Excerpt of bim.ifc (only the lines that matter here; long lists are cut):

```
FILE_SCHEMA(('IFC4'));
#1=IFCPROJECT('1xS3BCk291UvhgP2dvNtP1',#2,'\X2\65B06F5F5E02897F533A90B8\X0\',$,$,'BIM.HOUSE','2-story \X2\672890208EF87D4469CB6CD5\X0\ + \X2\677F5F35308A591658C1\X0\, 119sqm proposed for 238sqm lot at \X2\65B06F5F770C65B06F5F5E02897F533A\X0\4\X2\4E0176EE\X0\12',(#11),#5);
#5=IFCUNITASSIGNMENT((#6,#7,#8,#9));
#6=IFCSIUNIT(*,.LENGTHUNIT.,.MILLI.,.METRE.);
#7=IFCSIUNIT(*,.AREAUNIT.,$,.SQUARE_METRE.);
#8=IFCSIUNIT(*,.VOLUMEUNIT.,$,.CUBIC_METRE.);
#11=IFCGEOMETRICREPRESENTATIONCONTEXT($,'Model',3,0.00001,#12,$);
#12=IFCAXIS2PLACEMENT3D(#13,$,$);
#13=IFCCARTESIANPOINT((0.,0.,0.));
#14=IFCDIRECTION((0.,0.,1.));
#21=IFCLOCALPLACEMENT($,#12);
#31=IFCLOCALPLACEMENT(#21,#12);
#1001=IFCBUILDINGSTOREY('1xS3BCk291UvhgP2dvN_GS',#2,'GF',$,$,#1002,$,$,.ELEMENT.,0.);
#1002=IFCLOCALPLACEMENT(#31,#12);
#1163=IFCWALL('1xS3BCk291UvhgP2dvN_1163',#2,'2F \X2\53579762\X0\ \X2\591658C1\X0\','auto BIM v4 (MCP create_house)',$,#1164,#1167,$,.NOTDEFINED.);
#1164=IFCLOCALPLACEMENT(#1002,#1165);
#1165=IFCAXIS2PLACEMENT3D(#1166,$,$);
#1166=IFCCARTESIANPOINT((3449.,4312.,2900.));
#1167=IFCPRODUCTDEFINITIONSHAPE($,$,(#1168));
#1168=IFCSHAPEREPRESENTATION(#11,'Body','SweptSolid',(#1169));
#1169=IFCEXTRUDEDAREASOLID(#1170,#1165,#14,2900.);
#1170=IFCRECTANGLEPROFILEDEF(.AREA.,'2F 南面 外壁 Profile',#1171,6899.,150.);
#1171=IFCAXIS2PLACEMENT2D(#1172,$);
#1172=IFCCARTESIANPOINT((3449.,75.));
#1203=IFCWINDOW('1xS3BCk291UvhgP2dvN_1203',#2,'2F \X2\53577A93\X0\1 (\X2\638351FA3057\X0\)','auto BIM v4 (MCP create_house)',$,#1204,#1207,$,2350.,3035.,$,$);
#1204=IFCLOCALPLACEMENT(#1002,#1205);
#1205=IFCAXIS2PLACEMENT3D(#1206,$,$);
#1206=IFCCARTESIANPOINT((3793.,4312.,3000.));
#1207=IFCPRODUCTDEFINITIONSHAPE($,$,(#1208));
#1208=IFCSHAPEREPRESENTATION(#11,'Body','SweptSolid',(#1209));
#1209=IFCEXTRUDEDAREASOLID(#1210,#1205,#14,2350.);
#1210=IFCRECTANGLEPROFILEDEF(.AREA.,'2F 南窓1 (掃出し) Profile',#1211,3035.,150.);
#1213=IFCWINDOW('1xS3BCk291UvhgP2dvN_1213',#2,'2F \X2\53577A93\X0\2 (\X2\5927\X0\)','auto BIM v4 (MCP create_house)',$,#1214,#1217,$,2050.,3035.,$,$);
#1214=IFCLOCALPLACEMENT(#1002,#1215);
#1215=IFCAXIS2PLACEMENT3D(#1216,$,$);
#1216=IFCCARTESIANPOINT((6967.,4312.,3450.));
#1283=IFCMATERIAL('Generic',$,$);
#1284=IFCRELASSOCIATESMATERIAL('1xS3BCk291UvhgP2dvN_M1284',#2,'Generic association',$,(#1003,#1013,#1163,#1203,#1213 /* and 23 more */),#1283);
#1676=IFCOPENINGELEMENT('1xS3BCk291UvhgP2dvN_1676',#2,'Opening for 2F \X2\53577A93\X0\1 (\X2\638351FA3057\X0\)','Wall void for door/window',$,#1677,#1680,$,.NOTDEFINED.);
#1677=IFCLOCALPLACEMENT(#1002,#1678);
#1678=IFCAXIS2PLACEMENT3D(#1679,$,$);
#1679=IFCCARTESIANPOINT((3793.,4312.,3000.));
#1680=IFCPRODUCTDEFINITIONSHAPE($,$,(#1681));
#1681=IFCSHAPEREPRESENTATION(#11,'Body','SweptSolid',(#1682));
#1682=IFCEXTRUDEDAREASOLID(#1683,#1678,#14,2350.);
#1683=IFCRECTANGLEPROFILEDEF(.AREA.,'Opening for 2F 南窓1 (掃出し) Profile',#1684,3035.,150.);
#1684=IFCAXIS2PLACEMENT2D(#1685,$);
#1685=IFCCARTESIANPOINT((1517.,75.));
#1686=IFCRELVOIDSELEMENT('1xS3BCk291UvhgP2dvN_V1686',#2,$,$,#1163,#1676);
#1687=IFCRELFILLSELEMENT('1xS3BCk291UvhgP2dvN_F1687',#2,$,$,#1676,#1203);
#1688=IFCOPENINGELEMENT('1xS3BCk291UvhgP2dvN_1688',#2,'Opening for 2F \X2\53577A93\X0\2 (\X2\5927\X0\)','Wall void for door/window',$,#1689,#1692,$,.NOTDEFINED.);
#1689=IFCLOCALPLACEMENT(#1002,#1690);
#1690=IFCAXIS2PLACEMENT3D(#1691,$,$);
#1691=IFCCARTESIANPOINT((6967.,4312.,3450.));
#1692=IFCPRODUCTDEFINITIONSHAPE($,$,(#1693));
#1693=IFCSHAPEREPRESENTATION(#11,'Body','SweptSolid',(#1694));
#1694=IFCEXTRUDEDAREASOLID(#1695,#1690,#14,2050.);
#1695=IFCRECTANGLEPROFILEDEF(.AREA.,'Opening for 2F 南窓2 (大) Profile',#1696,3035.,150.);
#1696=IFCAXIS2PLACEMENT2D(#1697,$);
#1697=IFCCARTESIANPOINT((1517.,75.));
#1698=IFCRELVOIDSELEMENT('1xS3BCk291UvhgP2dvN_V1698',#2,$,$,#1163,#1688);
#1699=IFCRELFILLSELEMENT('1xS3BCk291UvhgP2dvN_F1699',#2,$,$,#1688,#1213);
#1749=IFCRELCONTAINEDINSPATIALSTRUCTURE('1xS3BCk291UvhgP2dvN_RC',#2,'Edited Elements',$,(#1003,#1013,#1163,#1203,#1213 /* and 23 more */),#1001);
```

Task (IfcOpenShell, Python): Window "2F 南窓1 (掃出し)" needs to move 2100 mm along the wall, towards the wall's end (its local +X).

```python
import ifcopenshell
import ifcopenshell.api.geometry
import ifcopenshell.util.placement
import ifcopenshell.util.unit

model = ifcopenshell.open("bim.ifc")
unit_scale = ifcopenshell.util.unit.calculate_unit_scale(model)

window = model.by_guid("1xS3BCk291UvhgP2dvN_1203")
opening = window.FillsVoids[0].RelatingOpeningElement
wall = opening.VoidsElements[0].RelatingBuildingElement

wall_matrix = ifcopenshell.util.placement.get_local_placement(wall.ObjectPlacement)
shift = wall_matrix[:3, 0] * 2.1 / unit_scale
before = ifcopenshell.util.placement.get_local_placement(window.ObjectPlacement)[:3, 3].copy()

# The window is not placed relative to its opening, so move both.
for product in (opening, window):
    matrix = ifcopenshell.util.placement.get_local_placement(product.ObjectPlacement)
    matrix[:3, 3] += shift
    ifcopenshell.api.geometry.edit_object_placement(model, product=product, matrix=matrix, is_si=False)

after = ifcopenshell.util.placement.get_local_placement(window.ObjectPlacement)[:3, 3]
print("window moved by", (after - before).round(3) + 0.0)

model.write("bim_updated.ifc")
```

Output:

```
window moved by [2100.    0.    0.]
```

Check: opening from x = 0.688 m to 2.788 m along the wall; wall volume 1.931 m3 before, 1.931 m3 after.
